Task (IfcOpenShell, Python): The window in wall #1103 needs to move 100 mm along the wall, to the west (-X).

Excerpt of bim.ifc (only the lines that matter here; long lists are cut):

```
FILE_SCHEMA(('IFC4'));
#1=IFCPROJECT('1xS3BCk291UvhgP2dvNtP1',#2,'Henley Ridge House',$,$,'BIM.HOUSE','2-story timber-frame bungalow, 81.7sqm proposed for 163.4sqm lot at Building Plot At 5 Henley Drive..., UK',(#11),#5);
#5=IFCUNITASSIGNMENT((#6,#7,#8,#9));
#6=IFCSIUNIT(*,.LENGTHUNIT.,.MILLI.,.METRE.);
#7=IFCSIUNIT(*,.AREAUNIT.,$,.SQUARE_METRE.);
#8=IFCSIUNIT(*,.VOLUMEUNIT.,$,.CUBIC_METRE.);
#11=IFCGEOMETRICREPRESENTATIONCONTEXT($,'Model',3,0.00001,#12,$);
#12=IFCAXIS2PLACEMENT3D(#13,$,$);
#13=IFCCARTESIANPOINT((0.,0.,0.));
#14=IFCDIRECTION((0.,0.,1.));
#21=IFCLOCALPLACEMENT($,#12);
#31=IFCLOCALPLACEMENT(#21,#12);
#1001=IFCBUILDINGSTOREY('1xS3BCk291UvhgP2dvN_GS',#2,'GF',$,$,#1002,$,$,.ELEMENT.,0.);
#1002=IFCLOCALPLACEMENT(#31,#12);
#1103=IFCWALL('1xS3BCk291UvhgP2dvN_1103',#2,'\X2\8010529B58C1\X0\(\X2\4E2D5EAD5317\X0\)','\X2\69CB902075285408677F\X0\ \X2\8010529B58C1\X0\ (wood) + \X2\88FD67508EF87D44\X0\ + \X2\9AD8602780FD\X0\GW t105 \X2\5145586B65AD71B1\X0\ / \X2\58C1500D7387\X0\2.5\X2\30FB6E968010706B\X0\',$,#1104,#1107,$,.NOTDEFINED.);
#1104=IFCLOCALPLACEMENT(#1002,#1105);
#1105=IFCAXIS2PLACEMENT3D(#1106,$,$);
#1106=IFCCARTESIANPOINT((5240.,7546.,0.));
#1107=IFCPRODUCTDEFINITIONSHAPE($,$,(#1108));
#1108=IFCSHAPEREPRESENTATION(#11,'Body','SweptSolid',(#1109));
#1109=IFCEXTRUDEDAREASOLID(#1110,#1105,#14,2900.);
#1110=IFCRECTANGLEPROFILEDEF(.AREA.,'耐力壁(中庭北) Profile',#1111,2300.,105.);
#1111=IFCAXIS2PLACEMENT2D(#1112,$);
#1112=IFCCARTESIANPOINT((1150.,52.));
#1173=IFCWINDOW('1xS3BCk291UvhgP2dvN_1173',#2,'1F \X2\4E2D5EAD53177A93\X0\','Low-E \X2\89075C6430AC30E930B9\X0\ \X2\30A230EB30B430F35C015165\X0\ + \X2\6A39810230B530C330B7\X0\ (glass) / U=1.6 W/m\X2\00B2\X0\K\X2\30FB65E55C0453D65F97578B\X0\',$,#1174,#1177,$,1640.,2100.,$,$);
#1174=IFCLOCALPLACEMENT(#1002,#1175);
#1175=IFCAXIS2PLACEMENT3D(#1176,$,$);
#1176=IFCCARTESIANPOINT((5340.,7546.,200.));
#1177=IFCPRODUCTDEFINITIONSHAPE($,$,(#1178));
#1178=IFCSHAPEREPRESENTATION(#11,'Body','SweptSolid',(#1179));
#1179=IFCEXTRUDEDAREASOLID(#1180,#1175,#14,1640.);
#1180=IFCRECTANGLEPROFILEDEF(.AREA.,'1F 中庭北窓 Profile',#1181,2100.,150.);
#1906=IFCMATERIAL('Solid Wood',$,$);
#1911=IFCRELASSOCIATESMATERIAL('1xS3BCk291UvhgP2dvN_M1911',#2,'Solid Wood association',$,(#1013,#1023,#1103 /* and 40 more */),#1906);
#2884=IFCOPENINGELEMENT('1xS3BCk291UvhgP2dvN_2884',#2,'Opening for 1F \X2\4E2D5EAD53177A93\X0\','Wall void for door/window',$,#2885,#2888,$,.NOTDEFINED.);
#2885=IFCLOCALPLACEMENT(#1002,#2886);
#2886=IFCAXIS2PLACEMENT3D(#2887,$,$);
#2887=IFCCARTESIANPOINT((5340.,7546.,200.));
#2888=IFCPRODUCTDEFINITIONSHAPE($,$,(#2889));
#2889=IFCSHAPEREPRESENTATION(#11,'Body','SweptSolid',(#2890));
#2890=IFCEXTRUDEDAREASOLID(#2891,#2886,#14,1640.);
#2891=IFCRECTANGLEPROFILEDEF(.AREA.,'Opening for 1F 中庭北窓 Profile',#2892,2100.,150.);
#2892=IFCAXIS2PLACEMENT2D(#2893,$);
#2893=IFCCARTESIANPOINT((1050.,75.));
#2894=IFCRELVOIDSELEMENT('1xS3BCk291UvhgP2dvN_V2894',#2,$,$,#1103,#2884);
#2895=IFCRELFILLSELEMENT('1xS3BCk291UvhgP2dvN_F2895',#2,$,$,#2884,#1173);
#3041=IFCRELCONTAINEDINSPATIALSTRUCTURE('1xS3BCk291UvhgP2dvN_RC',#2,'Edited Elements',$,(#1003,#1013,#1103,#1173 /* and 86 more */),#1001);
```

```python
import ifcopenshell
import ifcopenshell.api.geometry
import ifcopenshell.util.placement
import ifcopenshell.util.unit

model = ifcopenshell.open("bim.ifc")
unit_scale = ifcopenshell.util.unit.calculate_unit_scale(model)

window = model.by_id(1173)
opening = window.FillsVoids[0].RelatingOpeningElement
wall = opening.VoidsElements[0].RelatingBuildingElement

wall_matrix = ifcopenshell.util.placement.get_local_placement(wall.ObjectPlacement)
shift = wall_matrix[:3, 0] * -0.1 / unit_scale
before = ifcopenshell.util.placement.get_local_placement(window.ObjectPlacement)[:3, 3].copy()

# The window is not placed relative to its opening, so move both.
for product in (opening, window):
    matrix = ifcopenshell.util.placement.get_local_placement(product.ObjectPlacement)
    matrix[:3, 3] += shift
    ifcopenshell.api.geometry.edit_object_placement(model, product=product, matrix=matrix, is_si=False)

after = ifcopenshell.util.placement.get_local_placement(window.ObjectPlacement)[:3, 3]
print("window moved by", (after - before).round(3) + 0.0)

model.write("bim_edited.ifc")
```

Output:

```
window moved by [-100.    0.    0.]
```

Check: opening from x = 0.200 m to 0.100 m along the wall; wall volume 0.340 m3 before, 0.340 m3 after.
